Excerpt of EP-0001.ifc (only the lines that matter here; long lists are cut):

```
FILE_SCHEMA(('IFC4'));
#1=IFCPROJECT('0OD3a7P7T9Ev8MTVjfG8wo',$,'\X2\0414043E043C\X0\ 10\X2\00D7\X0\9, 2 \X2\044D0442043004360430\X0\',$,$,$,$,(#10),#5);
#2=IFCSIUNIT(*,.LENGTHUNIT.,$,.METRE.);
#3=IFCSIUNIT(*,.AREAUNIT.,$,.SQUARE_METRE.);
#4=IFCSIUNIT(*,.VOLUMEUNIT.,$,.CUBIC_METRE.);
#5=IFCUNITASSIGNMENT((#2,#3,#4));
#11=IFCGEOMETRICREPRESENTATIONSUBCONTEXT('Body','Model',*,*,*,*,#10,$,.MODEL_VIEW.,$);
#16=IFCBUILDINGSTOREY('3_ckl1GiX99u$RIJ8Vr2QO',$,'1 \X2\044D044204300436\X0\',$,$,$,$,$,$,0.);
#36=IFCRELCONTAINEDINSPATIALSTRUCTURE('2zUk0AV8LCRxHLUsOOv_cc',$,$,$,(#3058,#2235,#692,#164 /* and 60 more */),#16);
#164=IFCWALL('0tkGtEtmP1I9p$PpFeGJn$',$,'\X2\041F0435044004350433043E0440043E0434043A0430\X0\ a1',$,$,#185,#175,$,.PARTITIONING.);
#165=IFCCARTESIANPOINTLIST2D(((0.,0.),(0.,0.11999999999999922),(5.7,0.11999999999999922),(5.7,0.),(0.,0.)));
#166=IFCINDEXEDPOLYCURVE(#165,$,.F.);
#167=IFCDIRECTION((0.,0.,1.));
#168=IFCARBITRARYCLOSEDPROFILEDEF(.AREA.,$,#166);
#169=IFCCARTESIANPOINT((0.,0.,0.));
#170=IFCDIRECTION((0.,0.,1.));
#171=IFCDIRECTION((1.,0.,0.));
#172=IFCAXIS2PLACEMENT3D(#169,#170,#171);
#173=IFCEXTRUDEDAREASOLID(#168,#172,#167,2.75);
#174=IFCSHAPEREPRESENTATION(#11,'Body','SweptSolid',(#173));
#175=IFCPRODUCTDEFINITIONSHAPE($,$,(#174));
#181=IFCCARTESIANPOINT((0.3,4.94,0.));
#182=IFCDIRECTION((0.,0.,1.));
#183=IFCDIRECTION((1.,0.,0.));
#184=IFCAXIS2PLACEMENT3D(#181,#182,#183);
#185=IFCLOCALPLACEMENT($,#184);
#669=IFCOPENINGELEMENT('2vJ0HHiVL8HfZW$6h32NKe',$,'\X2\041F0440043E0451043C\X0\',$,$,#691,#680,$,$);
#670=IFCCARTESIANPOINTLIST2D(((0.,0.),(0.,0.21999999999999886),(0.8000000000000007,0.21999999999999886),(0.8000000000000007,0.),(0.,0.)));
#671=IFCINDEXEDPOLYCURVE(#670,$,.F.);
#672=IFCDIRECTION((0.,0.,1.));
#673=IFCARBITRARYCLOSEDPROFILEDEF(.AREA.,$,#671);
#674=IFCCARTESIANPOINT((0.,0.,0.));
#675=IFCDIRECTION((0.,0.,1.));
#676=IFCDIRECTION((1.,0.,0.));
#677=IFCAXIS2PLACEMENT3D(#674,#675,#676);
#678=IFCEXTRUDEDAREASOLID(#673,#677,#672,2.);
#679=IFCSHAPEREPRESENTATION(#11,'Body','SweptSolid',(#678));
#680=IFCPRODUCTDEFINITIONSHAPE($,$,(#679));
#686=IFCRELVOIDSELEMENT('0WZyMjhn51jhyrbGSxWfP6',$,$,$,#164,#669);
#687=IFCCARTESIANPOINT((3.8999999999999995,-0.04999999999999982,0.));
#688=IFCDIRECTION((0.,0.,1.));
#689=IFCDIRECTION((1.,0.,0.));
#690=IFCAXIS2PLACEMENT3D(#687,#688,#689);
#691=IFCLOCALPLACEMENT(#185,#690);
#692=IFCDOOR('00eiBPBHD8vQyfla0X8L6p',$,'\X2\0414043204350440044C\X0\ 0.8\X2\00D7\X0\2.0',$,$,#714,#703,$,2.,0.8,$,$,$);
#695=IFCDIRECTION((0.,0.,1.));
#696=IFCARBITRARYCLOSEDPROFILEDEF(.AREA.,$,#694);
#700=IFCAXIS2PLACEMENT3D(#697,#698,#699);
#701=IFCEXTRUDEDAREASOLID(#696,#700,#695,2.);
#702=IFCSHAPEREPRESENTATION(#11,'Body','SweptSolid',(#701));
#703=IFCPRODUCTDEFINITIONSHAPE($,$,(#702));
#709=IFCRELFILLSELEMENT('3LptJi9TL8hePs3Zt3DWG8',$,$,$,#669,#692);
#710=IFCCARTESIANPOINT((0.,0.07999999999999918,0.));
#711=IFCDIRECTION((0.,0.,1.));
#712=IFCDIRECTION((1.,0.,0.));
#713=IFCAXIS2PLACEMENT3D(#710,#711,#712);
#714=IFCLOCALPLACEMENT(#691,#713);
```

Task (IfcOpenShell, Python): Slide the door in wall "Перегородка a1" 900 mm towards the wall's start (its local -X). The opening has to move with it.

```python
import ifcopenshell
import ifcopenshell.api.geometry
import ifcopenshell.util.placement
import ifcopenshell.util.unit

model = ifcopenshell.open("EP-0001.ifc")
unit_scale = ifcopenshell.util.unit.calculate_unit_scale(model)

door = model.by_id(692)
opening = door.FillsVoids[0].RelatingOpeningElement
wall = opening.VoidsElements[0].RelatingBuildingElement

wall_matrix = ifcopenshell.util.placement.get_local_placement(wall.ObjectPlacement)
shift = wall_matrix[:3, 0] * -0.9 / unit_scale
before = ifcopenshell.util.placement.get_local_placement(door.ObjectPlacement)[:3, 3].copy()

# The door is placed relative to its opening, so it follows when the opening moves.
matrix = ifcopenshell.util.placement.get_local_placement(opening.ObjectPlacement)
matrix[:3, 3] += shift
ifcopenshell.api.geometry.edit_object_placement(
    model, product=opening, matrix=matrix, is_si=False, should_transform_children=True
)

after = ifcopenshell.util.placement.get_local_placement(door.ObjectPlacement)[:3, 3]
print("door moved by", (after - before).round(3) + 0.0)

model.write("EP-0001-out.ifc")
```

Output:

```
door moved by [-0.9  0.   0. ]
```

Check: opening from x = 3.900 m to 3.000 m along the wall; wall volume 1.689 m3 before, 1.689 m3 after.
